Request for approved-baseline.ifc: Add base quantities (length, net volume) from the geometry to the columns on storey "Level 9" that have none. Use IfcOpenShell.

First a look at what the model holds.

```python
import ifcopenshell
import ifcopenshell.util.element
import ifcopenshell.util.unit

model = ifcopenshell.open("approved-baseline.ifc")
print(model.schema)
for unit_type in ("LENGTHUNIT", "AREAUNIT", "VOLUMEUNIT"):
    print(unit_type, ifcopenshell.util.unit.calculate_unit_scale(model, unit_type))
storey = next(s for s in model.by_type("IfcBuildingStorey") if s.Name == "Level 9")
columns = [e for e in ifcopenshell.util.element.get_decomposition(storey) if e.is_a("IfcColumn")]
for e in sorted(columns, key=lambda e: e.id()):
    print(e.id(), e.is_a(), e.Name, list(ifcopenshell.util.element.get_psets(e, qtos_only=True)), sep=" | ")
```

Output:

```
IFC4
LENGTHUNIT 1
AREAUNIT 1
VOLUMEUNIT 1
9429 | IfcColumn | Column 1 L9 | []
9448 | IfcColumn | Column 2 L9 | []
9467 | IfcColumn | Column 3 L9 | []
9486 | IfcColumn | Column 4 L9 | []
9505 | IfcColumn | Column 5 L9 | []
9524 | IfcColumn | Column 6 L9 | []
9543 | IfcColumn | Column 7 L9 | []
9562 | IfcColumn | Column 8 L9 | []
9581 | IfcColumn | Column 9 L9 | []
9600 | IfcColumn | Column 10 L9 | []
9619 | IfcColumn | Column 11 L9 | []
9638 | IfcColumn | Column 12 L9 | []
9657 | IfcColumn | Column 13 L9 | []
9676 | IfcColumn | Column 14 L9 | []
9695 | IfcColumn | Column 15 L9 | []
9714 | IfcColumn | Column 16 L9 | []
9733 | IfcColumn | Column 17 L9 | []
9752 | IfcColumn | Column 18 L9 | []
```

```python
import ifcopenshell
import ifcopenshell.api.pset
import ifcopenshell.geom
import ifcopenshell.util.element
import ifcopenshell.util.shape
import ifcopenshell.util.unit

model = ifcopenshell.open("approved-baseline.ifc")
unit_scale = ifcopenshell.util.unit.calculate_unit_scale(model)
volume_scale = ifcopenshell.util.unit.calculate_unit_scale(model, "VOLUMEUNIT")
settings = ifcopenshell.geom.settings()

storey = next(s for s in model.by_type("IfcBuildingStorey") if s.Name == "Level 9")
columns = [e for e in ifcopenshell.util.element.get_decomposition(storey) if e.is_a("IfcColumn")]

for e in sorted(columns, key=lambda e: e.id()):
    if ifcopenshell.util.element.get_psets(e, qtos_only=True, should_inherit=False):
        continue
    # Geometry comes back in metres, in the element's own axes.
    shape = ifcopenshell.geom.create_shape(settings, e)
    values = {
        "Length": ifcopenshell.util.shape.get_z(shape.geometry) / unit_scale,
        "NetVolume": ifcopenshell.util.shape.get_volume(shape.geometry) / volume_scale,
    }
    qto = ifcopenshell.api.pset.add_qto(model, product=e, name="Qto_ColumnBaseQuantities")
    ifcopenshell.api.pset.edit_qto(model, qto=qto, properties=values)
    print(e.id(), {k: round(v, 3) for k, v in values.items()})

model.write("approved-baseline_v2.ifc")
```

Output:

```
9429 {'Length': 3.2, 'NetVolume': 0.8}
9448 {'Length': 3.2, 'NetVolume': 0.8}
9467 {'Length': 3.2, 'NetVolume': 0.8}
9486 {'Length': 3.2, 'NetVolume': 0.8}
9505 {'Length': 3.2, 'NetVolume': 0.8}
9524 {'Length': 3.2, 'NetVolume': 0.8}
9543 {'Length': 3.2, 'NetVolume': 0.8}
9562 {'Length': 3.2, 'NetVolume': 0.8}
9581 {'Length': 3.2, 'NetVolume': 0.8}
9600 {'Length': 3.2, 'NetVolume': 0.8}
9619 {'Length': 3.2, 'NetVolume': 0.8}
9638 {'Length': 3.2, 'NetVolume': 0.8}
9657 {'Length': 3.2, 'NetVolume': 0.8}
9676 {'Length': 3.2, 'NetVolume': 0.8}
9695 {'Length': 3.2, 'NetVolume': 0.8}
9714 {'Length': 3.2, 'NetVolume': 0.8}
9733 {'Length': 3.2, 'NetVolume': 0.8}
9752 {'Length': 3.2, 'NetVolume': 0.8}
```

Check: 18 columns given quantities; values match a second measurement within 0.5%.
